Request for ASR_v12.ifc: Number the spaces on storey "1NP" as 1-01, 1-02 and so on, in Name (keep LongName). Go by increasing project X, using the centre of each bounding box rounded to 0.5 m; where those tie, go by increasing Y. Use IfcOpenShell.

First a look at what the model holds.

```python
import ifcopenshell
import ifcopenshell.util.element
import ifcopenshell.util.placement

model = ifcopenshell.open("ASR_v12.ifc")
print(model.schema)
storey = next(s for s in model.by_type("IfcBuildingStorey") if s.Name == "1NP")
spaces = [e for e in ifcopenshell.util.element.get_decomposition(storey) if e.is_a("IfcSpace")]
for e in sorted(spaces, key=lambda e: e.id()):
    origin = ifcopenshell.util.placement.get_local_placement(e.ObjectPlacement)[:3, 3]
    print(e.id(), e.Name, e.LongName, origin.round(2) + 0.0, sep=" | ")
```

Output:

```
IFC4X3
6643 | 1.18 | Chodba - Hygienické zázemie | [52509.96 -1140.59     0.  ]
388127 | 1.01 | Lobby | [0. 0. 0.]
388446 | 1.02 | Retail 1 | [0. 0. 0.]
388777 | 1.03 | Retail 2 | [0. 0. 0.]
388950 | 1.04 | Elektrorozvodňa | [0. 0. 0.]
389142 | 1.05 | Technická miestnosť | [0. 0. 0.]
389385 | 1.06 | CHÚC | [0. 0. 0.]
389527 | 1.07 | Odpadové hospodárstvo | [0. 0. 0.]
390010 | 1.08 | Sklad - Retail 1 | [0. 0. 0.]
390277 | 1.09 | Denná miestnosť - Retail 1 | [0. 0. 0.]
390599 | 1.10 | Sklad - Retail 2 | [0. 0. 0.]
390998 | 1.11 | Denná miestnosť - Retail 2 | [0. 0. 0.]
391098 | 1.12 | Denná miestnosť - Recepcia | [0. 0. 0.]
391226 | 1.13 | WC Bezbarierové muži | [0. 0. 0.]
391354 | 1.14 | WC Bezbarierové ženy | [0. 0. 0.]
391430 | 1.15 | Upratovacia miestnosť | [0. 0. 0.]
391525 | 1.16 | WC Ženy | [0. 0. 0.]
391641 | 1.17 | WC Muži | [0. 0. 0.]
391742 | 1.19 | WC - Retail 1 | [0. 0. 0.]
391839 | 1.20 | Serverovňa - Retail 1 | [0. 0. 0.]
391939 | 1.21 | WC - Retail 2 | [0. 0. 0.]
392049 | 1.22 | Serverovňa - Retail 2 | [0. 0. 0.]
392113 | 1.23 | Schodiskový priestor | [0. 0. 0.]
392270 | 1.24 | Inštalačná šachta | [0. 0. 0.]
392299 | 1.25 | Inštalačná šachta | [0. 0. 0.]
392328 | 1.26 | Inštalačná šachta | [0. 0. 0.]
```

```python
import ifcopenshell
import ifcopenshell.geom
import ifcopenshell.util.element
import ifcopenshell.util.shape

model = ifcopenshell.open("ASR_v12.ifc")
settings = ifcopenshell.geom.settings()
settings.set("use-world-coords", True)


def centre(element):
    shape = ifcopenshell.geom.create_shape(settings, element)
    return ifcopenshell.util.shape.get_bbox_centroid(shape.geometry)


storey = next(s for s in model.by_type("IfcBuildingStorey") if s.Name == "1NP")
spaces = [e for e in ifcopenshell.util.element.get_decomposition(storey) if e.is_a("IfcSpace")]

# Insertion points can sit at a corner or the storey origin, so sort by the geometry (in metres).
centres = {e: centre(e) for e in spaces}
spaces.sort(key=lambda e: (round(centres[e][0] / 0.5), centres[e][1]))

for i, e in enumerate(spaces, start=1):
    number = f"1-{i:02d}"
    e.Name = number
    print(e.id(), number)

model.write("ASR_v12_edited.ifc")
```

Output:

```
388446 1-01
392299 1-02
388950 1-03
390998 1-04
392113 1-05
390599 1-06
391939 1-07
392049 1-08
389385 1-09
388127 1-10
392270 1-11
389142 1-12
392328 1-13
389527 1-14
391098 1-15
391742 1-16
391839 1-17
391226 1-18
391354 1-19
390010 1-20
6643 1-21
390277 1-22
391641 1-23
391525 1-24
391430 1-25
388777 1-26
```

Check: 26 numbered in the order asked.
